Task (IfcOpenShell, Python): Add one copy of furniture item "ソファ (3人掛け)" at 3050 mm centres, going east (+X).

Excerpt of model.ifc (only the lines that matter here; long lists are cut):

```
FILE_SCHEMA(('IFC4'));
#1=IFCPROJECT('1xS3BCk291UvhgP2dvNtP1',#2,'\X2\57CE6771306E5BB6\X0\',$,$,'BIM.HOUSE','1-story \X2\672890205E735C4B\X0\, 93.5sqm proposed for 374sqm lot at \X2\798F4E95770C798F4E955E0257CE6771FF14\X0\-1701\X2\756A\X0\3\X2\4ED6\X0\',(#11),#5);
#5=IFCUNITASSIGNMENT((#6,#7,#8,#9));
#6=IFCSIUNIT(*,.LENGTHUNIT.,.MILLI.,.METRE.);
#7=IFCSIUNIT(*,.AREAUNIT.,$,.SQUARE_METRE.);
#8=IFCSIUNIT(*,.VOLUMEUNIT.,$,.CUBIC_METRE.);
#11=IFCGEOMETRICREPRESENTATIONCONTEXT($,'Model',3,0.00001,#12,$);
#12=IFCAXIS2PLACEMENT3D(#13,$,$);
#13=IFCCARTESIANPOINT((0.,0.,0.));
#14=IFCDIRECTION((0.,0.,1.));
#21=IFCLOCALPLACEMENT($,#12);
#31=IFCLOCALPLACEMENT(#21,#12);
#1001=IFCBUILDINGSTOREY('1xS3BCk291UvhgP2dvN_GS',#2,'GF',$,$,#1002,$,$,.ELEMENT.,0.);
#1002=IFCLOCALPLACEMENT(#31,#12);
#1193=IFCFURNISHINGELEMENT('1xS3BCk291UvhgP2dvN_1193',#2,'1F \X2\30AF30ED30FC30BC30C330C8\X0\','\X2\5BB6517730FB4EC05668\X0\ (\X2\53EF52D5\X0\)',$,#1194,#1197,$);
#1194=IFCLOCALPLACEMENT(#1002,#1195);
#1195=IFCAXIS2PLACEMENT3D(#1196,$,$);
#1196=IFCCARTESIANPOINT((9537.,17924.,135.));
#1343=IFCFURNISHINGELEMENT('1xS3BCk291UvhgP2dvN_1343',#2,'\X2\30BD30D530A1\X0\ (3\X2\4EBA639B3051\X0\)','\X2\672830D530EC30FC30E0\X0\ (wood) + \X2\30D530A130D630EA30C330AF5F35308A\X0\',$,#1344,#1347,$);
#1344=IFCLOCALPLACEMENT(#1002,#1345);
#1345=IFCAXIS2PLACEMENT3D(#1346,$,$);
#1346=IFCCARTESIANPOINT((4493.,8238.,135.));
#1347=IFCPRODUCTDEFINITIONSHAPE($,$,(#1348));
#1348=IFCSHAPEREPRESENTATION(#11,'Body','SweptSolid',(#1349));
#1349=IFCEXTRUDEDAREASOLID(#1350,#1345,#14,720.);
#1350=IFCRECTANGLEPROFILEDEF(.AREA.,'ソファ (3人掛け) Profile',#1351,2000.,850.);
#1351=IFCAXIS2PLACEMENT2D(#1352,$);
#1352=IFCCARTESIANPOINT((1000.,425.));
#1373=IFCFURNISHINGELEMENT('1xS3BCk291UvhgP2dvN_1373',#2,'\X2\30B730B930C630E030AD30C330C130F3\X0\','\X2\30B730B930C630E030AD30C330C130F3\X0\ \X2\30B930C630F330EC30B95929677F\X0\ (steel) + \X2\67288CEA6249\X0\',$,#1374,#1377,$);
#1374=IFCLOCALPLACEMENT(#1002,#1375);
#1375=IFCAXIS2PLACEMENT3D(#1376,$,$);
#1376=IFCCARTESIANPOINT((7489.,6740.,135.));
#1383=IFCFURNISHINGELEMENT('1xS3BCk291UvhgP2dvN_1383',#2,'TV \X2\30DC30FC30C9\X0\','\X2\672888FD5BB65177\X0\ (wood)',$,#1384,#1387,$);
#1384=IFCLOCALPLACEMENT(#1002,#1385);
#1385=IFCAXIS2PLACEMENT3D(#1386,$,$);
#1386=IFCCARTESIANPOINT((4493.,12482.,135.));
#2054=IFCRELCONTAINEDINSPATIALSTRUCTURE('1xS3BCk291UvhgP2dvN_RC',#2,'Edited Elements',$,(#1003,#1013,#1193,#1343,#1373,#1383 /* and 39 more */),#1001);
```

```python
import numpy as np
import ifcopenshell
import ifcopenshell.api.geometry
import ifcopenshell.api.root
import ifcopenshell.util.element
import ifcopenshell.util.placement

model = ifcopenshell.open("model.ifc")


def reuse_history(source, copy):
    """copy_class also copies each property set's owner history, people and application; keep the originals."""
    for rel in copy.IsDefinedBy:
        if rel.is_a("IfcRelDefinesByProperties") and (history := rel.RelatingPropertyDefinition.OwnerHistory):
            rel.RelatingPropertyDefinition.OwnerHistory = source.OwnerHistory
            ifcopenshell.util.element.remove_deep2(model, history)


source = model.by_guid("1xS3BCk291UvhgP2dvN_1343")
base = ifcopenshell.util.placement.get_local_placement(source.ObjectPlacement)
step = np.array([1.0, 0.0, 0.0]) * 3050.0

for i in range(1, 2):
    copy = ifcopenshell.api.root.copy_class(model, product=source)
    copy.Representation = ifcopenshell.util.element.copy_deep(
        model, source.Representation, exclude=["IfcGeometricRepresentationContext", "IfcRepresentationMap"]
    )
    reuse_history(source, copy)
    matrix = base.copy()
    matrix[:3, 3] += i * step
    print("added at", matrix[:3, 3].round(3) + 0.0)
    ifcopenshell.api.geometry.edit_object_placement(model, product=copy, matrix=matrix, is_si=False)

model.write("model_updated.ifc")
```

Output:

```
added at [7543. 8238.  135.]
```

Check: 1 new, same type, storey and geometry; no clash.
